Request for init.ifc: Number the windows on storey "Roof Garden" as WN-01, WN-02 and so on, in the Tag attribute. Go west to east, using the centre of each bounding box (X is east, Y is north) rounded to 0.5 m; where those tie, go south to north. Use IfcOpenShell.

First a look at what the model holds.

```python
import ifcopenshell
import ifcopenshell.util.element
import ifcopenshell.util.placement

model = ifcopenshell.open("init.ifc")
print(model.schema)
storey = next(s for s in model.by_type("IfcBuildingStorey") if s.Name == "Roof Garden")
windows = [e for e in ifcopenshell.util.element.get_decomposition(storey) if e.is_a("IfcWindow")]
for e in sorted(windows, key=lambda e: e.id()):
    origin = ifcopenshell.util.placement.get_local_placement(e.ObjectPlacement)[:3, 3]
    print(e.id(), e.Tag, e.Name, origin.round(2) + 0.0, sep=" | ")
```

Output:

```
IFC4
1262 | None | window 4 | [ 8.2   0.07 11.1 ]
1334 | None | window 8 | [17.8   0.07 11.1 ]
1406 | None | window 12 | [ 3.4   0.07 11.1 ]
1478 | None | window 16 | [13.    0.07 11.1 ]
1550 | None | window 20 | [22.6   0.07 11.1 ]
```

```python
import ifcopenshell
import ifcopenshell.geom
import ifcopenshell.util.element
import ifcopenshell.util.shape

model = ifcopenshell.open("init.ifc")
settings = ifcopenshell.geom.settings()
settings.set("use-world-coords", True)


def centre(element):
    shape = ifcopenshell.geom.create_shape(settings, element)
    return ifcopenshell.util.shape.get_bbox_centroid(shape.geometry)


storey = next(s for s in model.by_type("IfcBuildingStorey") if s.Name == "Roof Garden")
windows = [e for e in ifcopenshell.util.element.get_decomposition(storey) if e.is_a("IfcWindow")]

# Insertion points can sit at a corner or the storey origin, so sort by the geometry (in metres).
centres = {e: centre(e) for e in windows}
windows.sort(key=lambda e: (round(centres[e][0] / 0.5), centres[e][1]))

for i, e in enumerate(windows, start=1):
    number = f"WN-{i:02d}"
    e.Tag = number
    print(e.id(), number)

model.write("init_edited.ifc")
```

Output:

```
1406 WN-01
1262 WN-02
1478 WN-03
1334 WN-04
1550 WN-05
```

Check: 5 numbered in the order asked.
